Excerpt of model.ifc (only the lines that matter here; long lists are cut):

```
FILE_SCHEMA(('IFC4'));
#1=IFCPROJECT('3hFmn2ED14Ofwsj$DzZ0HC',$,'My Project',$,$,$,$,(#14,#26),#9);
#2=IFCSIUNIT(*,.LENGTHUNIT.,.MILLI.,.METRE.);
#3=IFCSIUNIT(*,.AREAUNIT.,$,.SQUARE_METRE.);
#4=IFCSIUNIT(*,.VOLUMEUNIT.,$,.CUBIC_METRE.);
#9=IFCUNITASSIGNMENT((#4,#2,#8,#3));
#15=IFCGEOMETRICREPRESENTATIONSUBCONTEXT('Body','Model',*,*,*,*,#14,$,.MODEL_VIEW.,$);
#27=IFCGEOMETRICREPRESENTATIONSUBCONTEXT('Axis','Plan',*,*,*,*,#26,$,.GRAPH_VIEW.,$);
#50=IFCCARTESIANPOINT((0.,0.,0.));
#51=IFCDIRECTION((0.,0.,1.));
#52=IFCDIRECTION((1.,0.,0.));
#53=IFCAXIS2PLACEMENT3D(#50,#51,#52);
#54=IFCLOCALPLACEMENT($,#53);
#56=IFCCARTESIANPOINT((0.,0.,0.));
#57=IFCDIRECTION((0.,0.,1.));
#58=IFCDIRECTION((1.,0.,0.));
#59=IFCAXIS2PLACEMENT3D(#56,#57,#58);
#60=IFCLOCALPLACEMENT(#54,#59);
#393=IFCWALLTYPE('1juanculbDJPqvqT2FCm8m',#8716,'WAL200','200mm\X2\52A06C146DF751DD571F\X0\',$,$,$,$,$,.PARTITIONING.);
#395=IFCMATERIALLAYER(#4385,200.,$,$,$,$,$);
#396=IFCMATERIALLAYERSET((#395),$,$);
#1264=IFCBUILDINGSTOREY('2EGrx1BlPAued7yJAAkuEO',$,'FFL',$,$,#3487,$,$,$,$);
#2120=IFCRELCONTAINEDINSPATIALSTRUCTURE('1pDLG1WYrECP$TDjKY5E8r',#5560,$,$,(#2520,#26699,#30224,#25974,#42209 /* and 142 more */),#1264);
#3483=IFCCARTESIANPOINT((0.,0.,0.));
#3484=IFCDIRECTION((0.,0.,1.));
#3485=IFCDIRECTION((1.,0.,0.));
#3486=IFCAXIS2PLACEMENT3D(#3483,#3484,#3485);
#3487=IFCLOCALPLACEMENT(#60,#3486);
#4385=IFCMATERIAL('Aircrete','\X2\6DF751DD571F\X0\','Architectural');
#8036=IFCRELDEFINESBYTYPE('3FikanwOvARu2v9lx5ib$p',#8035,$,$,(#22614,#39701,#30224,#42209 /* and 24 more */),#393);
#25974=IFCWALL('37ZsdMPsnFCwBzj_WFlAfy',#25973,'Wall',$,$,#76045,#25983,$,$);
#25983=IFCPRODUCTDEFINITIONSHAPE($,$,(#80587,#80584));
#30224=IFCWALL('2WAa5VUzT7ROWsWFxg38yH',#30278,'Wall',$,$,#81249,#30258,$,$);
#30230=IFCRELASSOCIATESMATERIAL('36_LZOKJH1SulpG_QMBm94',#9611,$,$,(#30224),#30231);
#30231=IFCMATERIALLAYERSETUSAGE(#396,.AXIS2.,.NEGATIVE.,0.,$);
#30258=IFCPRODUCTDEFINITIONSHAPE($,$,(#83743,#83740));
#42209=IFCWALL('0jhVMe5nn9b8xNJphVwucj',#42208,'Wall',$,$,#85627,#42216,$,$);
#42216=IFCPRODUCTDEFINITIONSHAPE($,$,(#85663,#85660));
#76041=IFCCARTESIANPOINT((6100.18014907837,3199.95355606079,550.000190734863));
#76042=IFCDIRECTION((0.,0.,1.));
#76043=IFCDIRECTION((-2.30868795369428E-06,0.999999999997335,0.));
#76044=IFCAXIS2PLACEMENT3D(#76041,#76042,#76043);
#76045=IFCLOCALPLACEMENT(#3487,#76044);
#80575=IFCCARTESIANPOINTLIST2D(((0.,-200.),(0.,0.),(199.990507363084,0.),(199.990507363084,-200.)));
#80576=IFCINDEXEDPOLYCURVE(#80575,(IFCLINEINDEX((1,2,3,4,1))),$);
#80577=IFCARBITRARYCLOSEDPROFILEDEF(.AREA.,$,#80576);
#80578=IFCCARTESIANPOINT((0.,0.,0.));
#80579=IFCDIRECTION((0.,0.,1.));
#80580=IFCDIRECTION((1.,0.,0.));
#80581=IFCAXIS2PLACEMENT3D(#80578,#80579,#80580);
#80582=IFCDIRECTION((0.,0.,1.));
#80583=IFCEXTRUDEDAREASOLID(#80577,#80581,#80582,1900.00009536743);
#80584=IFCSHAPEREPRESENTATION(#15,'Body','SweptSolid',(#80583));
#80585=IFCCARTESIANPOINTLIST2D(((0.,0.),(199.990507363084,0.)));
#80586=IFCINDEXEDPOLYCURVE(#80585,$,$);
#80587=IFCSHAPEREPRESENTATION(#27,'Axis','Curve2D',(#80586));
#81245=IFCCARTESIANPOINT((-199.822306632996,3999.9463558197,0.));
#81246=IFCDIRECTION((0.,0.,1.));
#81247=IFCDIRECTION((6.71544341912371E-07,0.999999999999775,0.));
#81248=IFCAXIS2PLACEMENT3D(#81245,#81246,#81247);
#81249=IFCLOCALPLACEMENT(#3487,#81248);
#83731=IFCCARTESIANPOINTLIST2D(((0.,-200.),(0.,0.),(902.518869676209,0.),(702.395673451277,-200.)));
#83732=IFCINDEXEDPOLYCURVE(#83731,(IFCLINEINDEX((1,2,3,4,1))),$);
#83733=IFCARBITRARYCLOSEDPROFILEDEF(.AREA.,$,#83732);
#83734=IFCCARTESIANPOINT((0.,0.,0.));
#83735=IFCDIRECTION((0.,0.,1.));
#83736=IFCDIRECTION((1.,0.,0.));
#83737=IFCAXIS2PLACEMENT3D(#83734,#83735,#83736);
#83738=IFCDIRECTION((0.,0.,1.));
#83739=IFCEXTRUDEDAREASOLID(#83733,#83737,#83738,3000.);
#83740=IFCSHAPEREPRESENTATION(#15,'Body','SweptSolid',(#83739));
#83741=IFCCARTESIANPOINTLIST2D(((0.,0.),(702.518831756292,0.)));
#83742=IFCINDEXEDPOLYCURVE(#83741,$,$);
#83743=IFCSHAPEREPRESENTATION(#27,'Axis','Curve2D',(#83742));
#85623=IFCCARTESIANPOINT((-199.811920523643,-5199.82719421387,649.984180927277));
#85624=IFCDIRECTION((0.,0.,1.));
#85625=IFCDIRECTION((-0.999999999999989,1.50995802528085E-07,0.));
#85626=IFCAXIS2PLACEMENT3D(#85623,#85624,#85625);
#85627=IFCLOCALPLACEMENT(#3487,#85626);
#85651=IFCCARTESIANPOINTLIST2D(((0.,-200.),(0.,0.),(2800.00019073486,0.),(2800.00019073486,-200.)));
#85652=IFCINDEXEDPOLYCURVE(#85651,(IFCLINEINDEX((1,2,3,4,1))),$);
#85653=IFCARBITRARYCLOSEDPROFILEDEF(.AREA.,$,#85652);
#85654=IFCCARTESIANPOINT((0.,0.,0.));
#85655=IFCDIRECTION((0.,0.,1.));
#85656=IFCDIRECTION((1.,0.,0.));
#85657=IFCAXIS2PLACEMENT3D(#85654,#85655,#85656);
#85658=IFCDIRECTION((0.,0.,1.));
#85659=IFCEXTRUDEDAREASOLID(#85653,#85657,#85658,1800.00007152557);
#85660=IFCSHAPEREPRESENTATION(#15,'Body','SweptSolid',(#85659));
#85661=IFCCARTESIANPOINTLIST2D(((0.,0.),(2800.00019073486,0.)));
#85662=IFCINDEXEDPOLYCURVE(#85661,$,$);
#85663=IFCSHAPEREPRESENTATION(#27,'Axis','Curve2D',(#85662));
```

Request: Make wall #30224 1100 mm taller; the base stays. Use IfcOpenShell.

```python
import ifcopenshell
import ifcopenshell.geom
import ifcopenshell.util.representation
import ifcopenshell.util.shape

model = ifcopenshell.open("model.ifc")
settings = ifcopenshell.geom.settings()


def volume(element):
    """Net volume in cubic metres, openings subtracted."""
    shape = ifcopenshell.geom.create_shape(settings, element)
    return ifcopenshell.util.shape.get_volume(shape.geometry)


wall = model.by_id(30224)
before = volume(wall)

body = ifcopenshell.util.representation.get_representation(wall, "Model", "Body")
solid = body.Items[0]
old_height = solid.Depth
solid.Depth += 1100.0
after = volume(wall)

print(f"height {old_height:g} -> {solid.Depth:g}, volume {before:.3f} -> {after:.3f} m3")

model.write("model_v2.ifc")
```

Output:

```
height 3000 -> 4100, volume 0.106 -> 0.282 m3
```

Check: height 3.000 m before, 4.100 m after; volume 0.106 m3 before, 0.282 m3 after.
